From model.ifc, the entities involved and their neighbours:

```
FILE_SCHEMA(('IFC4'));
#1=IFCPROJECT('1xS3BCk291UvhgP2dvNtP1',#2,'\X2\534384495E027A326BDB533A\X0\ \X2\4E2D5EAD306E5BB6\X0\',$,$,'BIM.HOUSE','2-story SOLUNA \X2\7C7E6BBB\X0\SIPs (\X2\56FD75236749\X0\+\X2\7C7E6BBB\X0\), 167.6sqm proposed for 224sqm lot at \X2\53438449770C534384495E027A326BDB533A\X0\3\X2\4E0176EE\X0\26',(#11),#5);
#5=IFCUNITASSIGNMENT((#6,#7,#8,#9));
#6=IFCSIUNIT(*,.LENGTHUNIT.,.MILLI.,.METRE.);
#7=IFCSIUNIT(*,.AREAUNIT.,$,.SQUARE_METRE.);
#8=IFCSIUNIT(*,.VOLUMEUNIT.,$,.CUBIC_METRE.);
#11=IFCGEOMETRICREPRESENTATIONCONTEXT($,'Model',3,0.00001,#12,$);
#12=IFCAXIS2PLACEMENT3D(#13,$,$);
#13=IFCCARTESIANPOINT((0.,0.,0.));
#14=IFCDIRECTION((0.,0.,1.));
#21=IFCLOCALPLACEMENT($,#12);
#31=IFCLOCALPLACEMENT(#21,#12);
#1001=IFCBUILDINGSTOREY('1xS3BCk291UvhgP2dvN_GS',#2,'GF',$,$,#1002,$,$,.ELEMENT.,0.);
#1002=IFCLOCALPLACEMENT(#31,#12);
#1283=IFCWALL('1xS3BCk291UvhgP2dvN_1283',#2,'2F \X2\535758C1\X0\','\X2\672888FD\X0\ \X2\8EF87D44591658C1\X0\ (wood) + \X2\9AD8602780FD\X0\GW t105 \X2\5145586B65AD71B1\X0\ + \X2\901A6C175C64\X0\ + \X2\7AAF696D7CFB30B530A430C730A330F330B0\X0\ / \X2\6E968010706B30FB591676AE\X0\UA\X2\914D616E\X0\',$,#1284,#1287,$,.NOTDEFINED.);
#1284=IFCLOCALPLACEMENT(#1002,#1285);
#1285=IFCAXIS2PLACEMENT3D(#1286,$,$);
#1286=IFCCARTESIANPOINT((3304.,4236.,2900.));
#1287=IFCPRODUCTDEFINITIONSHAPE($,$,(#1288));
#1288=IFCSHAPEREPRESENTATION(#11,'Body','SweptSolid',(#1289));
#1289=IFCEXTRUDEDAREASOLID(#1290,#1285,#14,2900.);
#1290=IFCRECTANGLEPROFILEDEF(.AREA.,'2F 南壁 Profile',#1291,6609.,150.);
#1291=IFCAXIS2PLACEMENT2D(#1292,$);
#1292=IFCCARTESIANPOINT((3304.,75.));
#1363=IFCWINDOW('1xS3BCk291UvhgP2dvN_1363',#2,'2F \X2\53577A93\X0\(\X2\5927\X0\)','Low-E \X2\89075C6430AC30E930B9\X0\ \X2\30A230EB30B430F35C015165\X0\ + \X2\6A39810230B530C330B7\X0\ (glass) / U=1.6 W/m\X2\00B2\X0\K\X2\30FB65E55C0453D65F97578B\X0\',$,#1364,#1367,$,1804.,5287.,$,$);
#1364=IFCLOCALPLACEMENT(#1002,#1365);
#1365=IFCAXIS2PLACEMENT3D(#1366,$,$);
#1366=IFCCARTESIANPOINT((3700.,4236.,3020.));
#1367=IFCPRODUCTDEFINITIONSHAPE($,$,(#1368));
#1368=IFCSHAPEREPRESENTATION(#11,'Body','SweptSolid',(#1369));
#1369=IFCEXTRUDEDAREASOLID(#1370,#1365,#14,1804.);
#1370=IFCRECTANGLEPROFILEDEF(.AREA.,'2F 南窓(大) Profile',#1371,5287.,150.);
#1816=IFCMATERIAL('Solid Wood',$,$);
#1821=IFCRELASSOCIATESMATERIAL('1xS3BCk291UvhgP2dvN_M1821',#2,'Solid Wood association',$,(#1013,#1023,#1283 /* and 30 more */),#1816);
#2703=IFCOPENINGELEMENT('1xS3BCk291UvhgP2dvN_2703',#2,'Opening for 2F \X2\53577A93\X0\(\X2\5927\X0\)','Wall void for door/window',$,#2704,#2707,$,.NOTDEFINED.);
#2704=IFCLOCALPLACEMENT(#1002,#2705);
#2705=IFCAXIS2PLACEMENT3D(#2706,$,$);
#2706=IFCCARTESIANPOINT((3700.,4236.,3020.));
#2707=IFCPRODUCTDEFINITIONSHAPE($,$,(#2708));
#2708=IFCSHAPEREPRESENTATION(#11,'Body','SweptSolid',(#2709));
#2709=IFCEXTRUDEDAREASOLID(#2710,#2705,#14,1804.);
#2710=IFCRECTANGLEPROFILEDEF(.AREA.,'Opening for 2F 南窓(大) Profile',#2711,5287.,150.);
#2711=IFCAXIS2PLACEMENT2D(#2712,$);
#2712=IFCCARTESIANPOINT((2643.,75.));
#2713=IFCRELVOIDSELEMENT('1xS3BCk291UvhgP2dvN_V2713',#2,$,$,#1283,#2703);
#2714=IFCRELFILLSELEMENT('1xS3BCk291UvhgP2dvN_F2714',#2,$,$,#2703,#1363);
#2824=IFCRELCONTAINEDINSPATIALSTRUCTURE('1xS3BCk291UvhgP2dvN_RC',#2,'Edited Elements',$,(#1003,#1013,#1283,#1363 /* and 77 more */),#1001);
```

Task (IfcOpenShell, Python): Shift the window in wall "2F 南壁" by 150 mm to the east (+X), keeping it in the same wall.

```python
import ifcopenshell
import ifcopenshell.api.geometry
import ifcopenshell.util.placement

model = ifcopenshell.open("model.ifc")

window = model.by_guid("1xS3BCk291UvhgP2dvN_1363")
opening = window.FillsVoids[0].RelatingOpeningElement
wall = opening.VoidsElements[0].RelatingBuildingElement

wall_matrix = ifcopenshell.util.placement.get_local_placement(wall.ObjectPlacement)
shift = wall_matrix[:3, 0] * 150.0
before = ifcopenshell.util.placement.get_local_placement(window.ObjectPlacement)[:3, 3].copy()

# The window is not placed relative to its opening, so move both.
for product in (opening, window):
    matrix = ifcopenshell.util.placement.get_local_placement(product.ObjectPlacement)
    matrix[:3, 3] += shift
    ifcopenshell.api.geometry.edit_object_placement(model, product=product, matrix=matrix, is_si=False)

after = ifcopenshell.util.placement.get_local_placement(window.ObjectPlacement)[:3, 3]
print("window moved by", (after - before).round(3) + 0.0)

model.write("model_edited.ifc")
```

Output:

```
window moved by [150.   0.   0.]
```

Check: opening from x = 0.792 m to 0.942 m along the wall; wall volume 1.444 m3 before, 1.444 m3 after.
